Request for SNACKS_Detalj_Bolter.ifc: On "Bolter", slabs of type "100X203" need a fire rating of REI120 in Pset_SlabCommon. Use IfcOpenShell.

First a look at what the model holds.

```python
import ifcopenshell
import ifcopenshell.util.element

model = ifcopenshell.open("SNACKS_Detalj_Bolter.ifc")
print(model.schema)
storey = next(s for s in model.by_type("IfcBuildingStorey") if s.Name == "Bolter")
slabs = [e for e in ifcopenshell.util.element.get_decomposition(storey) if e.is_a("IfcSlab")]
seen = {}
for e in slabs:
    element_type = ifcopenshell.util.element.get_type(e)
    key = (element_type.Name if element_type != e and element_type else None, ifcopenshell.util.element.get_pset(e, "Pset_SlabCommon", "FireRating"))
    seen[key] = seen.get(key, 0) + 1
for (name, value), count in sorted(seen.items(), key=str):
    print(count, "x", name, "|", value)
```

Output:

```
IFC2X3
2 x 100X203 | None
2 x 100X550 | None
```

```python
import ifcopenshell
import ifcopenshell.api.pset
import ifcopenshell.util.element

model = ifcopenshell.open("SNACKS_Detalj_Bolter.ifc")

storey = next(s for s in model.by_type("IfcBuildingStorey") if s.Name == "Bolter")
slabs = [e for e in ifcopenshell.util.element.get_decomposition(storey) if e.is_a("IfcSlab")]

count = 0
for e in slabs:
    element_type = ifcopenshell.util.element.get_type(e)
    if element_type in (None, e) or element_type.Name != "100X203":
        continue
    # add_pset returns the element's existing set when there is one.
    pset = ifcopenshell.api.pset.add_pset(model, product=e, name="Pset_SlabCommon")
    ifcopenshell.api.pset.edit_pset(model, pset=pset, properties={"FireRating": "REI120"})
    count += 1

print(count, "slabs updated")

model.write("SNACKS_Detalj_Bolter-out.ifc")
```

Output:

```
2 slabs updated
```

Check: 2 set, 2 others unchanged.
